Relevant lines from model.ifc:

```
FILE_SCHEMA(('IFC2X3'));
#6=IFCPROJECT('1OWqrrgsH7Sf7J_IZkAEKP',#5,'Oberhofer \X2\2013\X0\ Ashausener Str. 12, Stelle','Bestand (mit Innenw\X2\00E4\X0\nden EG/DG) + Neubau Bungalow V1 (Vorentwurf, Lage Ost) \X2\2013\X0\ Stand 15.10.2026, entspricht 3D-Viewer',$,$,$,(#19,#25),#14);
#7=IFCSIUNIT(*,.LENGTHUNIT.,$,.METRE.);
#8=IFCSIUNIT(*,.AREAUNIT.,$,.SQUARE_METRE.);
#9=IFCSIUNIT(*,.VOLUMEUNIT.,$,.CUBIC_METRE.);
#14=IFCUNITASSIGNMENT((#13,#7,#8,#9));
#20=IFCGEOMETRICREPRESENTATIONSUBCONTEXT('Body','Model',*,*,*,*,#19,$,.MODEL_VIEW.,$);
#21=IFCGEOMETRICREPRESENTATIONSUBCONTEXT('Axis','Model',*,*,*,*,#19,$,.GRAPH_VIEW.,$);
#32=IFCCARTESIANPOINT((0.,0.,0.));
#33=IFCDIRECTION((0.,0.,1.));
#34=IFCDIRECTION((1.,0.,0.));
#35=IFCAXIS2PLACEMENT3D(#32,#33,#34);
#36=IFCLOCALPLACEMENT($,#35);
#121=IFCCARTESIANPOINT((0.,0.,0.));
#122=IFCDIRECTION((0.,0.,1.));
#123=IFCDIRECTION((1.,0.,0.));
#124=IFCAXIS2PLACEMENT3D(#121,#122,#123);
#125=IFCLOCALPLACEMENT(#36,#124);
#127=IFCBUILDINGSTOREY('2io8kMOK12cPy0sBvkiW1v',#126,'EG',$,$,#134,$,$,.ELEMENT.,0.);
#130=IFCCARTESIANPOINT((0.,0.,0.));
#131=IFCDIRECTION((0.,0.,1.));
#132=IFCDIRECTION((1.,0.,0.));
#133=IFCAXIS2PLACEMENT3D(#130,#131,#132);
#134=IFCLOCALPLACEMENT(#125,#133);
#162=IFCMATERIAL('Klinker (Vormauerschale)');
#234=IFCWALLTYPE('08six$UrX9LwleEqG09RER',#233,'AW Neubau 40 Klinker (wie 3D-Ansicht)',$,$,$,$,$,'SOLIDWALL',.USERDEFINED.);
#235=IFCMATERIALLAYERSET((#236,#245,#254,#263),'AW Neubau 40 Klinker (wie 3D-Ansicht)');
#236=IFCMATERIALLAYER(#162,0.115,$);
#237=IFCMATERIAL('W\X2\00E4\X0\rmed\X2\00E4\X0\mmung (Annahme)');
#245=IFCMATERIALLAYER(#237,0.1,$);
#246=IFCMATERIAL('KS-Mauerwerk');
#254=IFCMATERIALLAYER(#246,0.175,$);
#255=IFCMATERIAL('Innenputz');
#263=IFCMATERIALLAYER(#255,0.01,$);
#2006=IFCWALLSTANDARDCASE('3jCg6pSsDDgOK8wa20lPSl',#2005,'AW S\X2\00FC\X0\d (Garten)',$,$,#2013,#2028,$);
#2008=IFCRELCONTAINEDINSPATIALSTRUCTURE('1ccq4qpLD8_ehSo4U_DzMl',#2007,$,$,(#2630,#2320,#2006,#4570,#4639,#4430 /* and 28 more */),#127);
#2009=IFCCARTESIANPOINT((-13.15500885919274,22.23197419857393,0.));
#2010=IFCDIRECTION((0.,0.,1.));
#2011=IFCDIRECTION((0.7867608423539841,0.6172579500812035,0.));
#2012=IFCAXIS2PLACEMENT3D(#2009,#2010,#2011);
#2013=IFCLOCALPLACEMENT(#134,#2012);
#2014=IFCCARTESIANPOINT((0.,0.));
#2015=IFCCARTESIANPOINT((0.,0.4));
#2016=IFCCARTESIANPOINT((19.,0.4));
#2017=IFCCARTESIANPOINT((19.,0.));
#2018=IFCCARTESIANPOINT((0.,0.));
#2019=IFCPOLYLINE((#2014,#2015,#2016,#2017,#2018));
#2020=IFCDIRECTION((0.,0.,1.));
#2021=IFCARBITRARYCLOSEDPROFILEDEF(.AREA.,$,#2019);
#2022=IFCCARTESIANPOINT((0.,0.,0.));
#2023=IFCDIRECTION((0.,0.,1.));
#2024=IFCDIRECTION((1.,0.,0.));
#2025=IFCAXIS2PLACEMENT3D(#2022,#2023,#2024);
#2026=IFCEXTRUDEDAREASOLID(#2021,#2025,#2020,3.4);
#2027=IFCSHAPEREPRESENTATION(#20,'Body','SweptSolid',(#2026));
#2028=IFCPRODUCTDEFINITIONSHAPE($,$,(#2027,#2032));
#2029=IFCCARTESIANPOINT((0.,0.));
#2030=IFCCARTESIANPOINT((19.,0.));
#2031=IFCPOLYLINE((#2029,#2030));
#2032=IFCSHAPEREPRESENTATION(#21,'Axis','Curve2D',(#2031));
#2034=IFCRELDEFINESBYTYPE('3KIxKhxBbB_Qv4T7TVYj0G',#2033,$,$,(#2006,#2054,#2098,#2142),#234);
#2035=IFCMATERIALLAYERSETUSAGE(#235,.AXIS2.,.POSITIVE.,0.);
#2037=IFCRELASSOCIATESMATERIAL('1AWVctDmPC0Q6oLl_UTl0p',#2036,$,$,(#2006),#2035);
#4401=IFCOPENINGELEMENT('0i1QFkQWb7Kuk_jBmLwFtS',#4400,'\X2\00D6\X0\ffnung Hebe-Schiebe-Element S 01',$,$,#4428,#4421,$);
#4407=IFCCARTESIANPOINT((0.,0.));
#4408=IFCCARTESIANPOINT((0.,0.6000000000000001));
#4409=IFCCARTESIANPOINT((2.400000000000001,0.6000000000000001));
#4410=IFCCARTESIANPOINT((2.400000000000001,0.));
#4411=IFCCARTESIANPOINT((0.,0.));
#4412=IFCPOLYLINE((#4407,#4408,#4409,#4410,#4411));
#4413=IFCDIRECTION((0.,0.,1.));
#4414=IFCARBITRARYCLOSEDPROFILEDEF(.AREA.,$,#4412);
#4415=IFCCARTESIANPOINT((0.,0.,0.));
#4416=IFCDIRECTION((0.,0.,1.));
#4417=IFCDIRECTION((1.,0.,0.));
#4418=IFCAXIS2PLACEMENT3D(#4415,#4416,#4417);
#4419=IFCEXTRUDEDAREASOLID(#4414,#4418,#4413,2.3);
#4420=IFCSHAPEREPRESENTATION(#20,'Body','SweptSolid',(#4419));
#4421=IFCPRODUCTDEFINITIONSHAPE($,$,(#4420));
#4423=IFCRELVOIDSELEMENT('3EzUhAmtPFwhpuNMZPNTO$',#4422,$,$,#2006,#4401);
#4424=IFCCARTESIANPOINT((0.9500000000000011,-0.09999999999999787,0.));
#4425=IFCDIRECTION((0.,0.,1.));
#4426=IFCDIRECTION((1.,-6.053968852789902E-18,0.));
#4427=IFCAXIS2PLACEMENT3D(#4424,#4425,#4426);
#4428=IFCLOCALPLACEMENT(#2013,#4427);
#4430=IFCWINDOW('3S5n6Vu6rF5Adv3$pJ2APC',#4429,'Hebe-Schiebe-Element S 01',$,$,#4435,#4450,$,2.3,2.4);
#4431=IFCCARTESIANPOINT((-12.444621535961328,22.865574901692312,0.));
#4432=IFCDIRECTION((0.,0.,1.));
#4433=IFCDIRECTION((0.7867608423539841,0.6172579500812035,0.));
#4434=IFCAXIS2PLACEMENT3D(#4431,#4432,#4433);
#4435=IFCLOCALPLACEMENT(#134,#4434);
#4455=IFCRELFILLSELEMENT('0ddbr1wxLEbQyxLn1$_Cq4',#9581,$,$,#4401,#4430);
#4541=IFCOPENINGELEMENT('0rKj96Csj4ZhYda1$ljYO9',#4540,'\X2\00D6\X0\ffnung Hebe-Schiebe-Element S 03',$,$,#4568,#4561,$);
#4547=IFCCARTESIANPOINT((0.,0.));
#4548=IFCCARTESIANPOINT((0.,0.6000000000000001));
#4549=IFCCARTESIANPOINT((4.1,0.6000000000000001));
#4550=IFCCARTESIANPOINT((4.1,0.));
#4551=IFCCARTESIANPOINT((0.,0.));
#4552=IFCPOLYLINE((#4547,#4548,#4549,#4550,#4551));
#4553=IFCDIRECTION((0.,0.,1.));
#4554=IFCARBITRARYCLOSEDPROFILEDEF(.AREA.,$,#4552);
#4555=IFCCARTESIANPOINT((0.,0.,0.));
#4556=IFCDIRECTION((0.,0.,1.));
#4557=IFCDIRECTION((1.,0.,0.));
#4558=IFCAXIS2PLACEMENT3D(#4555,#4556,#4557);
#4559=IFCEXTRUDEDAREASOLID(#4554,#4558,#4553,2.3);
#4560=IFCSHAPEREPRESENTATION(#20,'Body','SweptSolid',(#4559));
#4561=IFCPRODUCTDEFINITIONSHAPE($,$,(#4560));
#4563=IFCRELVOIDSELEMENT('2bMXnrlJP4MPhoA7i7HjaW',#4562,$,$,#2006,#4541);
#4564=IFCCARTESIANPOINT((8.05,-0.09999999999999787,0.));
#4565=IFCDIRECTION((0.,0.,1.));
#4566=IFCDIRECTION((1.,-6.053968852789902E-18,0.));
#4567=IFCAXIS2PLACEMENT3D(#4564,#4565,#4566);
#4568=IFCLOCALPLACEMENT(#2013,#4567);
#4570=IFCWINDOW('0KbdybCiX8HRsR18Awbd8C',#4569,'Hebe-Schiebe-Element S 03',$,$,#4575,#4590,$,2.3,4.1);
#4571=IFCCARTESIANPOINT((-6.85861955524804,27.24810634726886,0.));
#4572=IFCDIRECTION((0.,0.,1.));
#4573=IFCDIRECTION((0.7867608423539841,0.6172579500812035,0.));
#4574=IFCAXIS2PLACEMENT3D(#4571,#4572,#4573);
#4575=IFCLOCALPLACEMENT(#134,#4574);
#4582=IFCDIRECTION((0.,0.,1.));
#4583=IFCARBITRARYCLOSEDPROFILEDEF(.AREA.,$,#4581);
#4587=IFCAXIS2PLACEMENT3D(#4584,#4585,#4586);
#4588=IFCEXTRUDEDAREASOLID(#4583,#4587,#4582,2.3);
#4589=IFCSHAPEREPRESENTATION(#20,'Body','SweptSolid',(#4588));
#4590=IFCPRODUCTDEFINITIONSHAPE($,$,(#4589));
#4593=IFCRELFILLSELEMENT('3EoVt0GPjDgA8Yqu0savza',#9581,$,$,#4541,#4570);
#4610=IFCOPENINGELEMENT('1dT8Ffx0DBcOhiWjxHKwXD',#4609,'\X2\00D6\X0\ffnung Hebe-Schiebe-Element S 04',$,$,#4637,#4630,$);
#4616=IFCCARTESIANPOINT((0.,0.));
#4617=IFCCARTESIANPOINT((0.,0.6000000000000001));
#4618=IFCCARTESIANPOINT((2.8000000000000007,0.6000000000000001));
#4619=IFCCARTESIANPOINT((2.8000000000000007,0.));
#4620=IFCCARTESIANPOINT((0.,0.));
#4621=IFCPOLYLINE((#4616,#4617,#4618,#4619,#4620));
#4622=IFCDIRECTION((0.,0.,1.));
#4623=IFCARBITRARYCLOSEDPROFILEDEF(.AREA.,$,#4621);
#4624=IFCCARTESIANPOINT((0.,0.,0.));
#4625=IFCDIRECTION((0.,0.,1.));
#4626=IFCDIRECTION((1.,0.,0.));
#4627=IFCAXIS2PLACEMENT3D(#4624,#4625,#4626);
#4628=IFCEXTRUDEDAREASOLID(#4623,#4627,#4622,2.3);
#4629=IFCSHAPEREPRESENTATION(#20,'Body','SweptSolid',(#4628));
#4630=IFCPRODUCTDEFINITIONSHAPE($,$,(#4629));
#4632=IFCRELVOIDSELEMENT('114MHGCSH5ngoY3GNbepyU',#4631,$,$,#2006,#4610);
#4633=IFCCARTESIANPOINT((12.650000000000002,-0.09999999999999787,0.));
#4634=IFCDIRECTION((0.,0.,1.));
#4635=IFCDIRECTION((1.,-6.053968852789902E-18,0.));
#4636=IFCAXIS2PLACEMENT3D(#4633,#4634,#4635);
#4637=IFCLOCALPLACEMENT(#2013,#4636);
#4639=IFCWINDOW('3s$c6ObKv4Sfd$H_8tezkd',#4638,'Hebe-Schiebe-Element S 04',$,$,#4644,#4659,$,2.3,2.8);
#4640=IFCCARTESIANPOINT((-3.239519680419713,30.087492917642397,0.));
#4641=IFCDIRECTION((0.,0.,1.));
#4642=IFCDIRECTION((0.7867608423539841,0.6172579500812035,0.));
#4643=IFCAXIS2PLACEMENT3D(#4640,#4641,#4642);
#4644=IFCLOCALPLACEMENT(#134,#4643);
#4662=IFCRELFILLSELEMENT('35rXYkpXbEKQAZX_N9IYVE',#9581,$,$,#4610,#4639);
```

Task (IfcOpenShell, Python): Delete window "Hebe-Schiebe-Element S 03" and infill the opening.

```python
import ifcopenshell
import ifcopenshell.api.feature
import ifcopenshell.api.root
import ifcopenshell.geom
import ifcopenshell.util.shape

model = ifcopenshell.open("model.ifc")
settings = ifcopenshell.geom.settings()


def volume(element):
    """Net volume in cubic metres, openings subtracted."""
    shape = ifcopenshell.geom.create_shape(settings, element)
    return ifcopenshell.util.shape.get_volume(shape.geometry)


window = model.by_id(4570)
opening = window.FillsVoids[0].RelatingOpeningElement
wall = opening.VoidsElements[0].RelatingBuildingElement
before = volume(wall)

ifcopenshell.api.root.remove_product(model, product=window)
ifcopenshell.api.feature.remove_feature(model, feature=opening)

after = volume(wall)

print(f"wall volume {before:.3f} -> {after:.3f} m3")

model.write("model_rev.ifc")
```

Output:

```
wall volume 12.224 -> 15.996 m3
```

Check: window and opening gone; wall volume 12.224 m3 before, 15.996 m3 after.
